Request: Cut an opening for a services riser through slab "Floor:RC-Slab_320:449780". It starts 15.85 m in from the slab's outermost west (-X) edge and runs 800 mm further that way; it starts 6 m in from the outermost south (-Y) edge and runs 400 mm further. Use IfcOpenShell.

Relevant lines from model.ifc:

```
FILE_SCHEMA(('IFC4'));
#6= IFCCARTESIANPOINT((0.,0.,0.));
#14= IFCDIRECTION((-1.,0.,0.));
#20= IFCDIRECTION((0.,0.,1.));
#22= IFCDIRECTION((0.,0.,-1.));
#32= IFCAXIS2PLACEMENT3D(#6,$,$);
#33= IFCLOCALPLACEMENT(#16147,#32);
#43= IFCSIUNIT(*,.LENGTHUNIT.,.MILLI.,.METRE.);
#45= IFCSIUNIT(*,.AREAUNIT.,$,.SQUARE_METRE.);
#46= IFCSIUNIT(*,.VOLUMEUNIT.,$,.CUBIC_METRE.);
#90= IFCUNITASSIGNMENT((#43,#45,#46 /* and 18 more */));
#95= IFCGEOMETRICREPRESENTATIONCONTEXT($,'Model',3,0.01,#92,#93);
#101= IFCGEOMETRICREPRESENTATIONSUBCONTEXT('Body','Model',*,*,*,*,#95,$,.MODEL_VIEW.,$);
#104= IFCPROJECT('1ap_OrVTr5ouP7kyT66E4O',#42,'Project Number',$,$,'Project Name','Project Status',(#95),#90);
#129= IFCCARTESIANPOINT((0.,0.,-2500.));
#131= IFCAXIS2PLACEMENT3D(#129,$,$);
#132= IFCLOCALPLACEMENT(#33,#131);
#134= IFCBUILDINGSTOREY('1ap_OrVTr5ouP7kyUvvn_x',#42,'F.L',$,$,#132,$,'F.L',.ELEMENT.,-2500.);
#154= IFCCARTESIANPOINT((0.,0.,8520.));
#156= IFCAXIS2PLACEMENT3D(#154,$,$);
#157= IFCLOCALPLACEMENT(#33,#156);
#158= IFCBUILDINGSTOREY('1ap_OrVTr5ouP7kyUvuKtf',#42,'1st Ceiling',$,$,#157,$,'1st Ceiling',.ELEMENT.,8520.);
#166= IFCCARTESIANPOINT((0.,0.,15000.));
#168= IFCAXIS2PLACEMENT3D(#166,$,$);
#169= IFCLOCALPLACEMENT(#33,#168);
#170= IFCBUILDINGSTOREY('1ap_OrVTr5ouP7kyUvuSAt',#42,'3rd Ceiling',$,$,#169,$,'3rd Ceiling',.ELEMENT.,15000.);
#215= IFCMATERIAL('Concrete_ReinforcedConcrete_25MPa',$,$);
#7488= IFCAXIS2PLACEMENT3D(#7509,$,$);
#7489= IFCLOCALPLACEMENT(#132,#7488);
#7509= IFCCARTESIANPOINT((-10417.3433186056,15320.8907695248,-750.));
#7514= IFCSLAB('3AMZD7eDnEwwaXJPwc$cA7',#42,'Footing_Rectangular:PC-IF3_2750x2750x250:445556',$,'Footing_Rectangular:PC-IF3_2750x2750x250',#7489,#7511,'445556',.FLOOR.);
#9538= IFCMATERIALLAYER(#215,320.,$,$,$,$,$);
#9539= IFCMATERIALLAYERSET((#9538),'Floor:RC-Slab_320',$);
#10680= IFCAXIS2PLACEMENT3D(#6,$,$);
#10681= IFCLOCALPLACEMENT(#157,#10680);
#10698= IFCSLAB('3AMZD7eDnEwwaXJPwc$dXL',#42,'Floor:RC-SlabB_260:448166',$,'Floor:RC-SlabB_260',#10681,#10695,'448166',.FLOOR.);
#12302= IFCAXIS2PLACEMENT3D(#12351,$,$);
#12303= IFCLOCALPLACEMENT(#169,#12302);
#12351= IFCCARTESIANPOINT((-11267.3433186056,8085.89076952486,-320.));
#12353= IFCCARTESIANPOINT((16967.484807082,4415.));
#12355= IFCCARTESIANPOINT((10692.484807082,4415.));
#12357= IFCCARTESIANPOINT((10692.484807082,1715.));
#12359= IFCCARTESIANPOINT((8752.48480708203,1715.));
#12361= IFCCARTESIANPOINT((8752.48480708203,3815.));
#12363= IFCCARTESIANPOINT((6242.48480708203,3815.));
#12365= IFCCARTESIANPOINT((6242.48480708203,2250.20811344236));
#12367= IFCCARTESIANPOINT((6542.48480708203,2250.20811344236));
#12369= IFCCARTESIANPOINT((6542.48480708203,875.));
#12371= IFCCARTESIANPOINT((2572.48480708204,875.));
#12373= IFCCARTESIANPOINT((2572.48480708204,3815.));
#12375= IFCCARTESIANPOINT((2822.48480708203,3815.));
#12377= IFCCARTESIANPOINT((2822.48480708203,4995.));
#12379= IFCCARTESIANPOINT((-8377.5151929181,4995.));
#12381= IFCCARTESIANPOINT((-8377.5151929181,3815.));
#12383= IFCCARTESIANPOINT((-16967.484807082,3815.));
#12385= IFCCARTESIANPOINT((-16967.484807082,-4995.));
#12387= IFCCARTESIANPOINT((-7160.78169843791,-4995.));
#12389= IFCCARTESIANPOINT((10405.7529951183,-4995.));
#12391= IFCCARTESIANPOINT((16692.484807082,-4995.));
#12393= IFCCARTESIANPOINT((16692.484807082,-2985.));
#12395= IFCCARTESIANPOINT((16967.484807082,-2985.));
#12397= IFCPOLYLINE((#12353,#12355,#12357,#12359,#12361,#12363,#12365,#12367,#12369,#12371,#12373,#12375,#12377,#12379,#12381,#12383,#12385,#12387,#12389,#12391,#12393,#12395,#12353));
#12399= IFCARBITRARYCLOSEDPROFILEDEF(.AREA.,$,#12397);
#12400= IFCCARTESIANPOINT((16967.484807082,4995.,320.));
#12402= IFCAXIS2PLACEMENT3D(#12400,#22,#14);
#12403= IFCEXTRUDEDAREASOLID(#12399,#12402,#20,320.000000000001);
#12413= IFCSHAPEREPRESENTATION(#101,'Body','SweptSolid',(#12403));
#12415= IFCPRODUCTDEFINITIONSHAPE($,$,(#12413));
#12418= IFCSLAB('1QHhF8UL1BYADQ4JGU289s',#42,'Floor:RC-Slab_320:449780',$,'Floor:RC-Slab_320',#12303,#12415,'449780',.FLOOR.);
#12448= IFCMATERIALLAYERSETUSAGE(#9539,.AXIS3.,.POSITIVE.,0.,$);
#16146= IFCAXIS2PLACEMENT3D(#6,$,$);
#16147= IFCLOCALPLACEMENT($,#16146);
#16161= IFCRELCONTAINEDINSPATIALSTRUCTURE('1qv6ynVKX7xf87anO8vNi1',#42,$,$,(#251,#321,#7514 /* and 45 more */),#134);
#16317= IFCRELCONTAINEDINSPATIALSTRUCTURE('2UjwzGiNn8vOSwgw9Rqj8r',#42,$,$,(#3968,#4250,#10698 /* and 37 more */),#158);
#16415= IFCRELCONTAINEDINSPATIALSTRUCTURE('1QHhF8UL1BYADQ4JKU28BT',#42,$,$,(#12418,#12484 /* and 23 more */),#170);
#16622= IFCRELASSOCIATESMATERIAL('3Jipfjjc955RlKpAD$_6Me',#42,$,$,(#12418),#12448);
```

```python
import numpy as np
import ifcopenshell
import ifcopenshell.api.feature
import ifcopenshell.api.geometry
import ifcopenshell.api.root
import ifcopenshell.geom
import ifcopenshell.util.placement
import ifcopenshell.util.representation
import ifcopenshell.util.shape
import ifcopenshell.util.unit

model = ifcopenshell.open("model.ifc")
unit_scale = ifcopenshell.util.unit.calculate_unit_scale(model)
settings = ifcopenshell.geom.settings()


def volume(element):
    """Net volume in cubic metres, openings subtracted."""
    shape = ifcopenshell.geom.create_shape(settings, element)
    return ifcopenshell.util.shape.get_volume(shape.geometry)


slab = model.by_guid("1QHhF8UL1BYADQ4JGU289s")
before = volume(slab)

# Extent in the slab's own axes, in metres. The edges named are its -X and -Y sides.
slab_shape = ifcopenshell.geom.create_shape(settings, slab)
vertices = ifcopenshell.util.shape.get_vertices(slab_shape.geometry)
x_min, y_min, bottom = vertices.min(axis=0)
top = vertices[:, 2].max()

opening = ifcopenshell.api.root.create_entity(model, ifc_class="IfcOpeningElement", name="Services riser opening", predefined_type="OPENING")
context = ifcopenshell.util.representation.get_context(model, "Model", "Body", "MODEL_VIEW")
width, depth = 0.8, 0.4
outline = [(0.0, 0.0), (width, 0.0), (width, depth), (0.0, depth), (0.0, 0.0)]
# Overshoot both faces by 50 mm so the cut is clean.
shape = ifcopenshell.api.geometry.add_slab_representation(
    model, context=context, depth=top - bottom + 0.1, polyline=outline
)
ifcopenshell.api.geometry.assign_representation(model, product=opening, representation=shape)

matrix = ifcopenshell.util.placement.get_local_placement(slab.ObjectPlacement)
matrix[:, 3] = matrix @ np.append(np.array([x_min + 15.85, y_min + 6, bottom - 0.05]) / unit_scale, 1.0)
ifcopenshell.api.geometry.edit_object_placement(model, product=opening, matrix=matrix, is_si=False)
ifcopenshell.api.feature.add_feature(model, feature=opening, element=slab)

after = volume(slab)

print(f"slab volume {before:.3f} -> {after:.3f} m3")

model.write("model_updated.ifc")
```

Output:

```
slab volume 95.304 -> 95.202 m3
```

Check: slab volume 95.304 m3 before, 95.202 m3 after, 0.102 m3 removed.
